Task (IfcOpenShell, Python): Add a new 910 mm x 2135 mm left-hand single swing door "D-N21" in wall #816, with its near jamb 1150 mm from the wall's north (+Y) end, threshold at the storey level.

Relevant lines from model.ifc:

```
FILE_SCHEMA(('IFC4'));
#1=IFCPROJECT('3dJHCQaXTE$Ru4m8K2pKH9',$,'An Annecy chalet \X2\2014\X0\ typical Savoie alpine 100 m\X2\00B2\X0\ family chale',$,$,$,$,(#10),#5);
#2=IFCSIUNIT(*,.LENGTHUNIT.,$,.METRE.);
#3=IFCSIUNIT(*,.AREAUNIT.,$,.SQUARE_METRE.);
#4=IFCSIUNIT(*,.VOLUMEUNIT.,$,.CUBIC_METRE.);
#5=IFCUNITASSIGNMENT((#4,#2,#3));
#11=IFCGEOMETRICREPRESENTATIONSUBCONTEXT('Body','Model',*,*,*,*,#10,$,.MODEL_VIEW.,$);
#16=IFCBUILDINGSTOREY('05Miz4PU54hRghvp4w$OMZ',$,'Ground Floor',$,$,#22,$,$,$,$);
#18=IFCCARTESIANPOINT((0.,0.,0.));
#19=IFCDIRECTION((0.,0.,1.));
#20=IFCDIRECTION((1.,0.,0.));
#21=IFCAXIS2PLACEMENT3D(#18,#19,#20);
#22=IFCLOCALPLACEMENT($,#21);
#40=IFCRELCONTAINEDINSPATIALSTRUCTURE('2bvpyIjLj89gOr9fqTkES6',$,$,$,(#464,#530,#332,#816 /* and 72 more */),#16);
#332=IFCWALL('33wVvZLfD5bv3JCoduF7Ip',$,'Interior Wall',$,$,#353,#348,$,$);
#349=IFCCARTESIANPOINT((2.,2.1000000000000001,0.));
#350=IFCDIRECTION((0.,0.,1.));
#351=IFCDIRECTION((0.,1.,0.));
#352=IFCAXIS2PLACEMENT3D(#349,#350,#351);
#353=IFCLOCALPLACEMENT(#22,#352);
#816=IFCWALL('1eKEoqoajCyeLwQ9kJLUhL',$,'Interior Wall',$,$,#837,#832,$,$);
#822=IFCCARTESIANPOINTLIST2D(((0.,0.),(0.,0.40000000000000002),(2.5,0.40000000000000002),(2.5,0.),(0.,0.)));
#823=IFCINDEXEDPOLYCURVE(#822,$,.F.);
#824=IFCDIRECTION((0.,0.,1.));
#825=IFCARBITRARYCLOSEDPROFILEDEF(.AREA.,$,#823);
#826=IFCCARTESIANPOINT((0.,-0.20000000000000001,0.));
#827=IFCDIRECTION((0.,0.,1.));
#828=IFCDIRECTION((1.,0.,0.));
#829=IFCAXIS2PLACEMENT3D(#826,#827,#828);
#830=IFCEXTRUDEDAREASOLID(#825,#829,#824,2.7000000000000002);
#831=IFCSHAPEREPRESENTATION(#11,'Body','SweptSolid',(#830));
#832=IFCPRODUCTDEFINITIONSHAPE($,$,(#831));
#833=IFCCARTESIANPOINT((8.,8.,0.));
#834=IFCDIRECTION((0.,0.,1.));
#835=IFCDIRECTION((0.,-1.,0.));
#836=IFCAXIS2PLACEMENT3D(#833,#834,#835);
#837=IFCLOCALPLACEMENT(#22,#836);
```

```python
import numpy as np
import ifcopenshell
import ifcopenshell.api.feature
import ifcopenshell.api.geometry
import ifcopenshell.api.root
import ifcopenshell.api.spatial
import ifcopenshell.geom
import ifcopenshell.util.element
import ifcopenshell.util.placement
import ifcopenshell.util.representation
import ifcopenshell.util.shape
import ifcopenshell.util.unit

model = ifcopenshell.open("model.ifc")
unit_scale = ifcopenshell.util.unit.calculate_unit_scale(model)
settings = ifcopenshell.geom.settings()


def volume(element):
    """Net volume in cubic metres, openings subtracted."""
    shape = ifcopenshell.geom.create_shape(settings, element)
    return ifcopenshell.util.shape.get_volume(shape.geometry)


wall = model.by_guid("1eKEoqoajCyeLwQ9kJLUhL")
storey = ifcopenshell.util.element.get_container(wall, ifc_class="IfcBuildingStorey")
context = ifcopenshell.util.representation.get_context(model, "Model", "Body", "MODEL_VIEW")
before = volume(wall)

width, height, from_end, sill = 0.91, 2.135, 1.15, 0.0  # metres

# The wall runs along its own X axis, and the end named is its -X end.
wall_shape = ifcopenshell.geom.create_shape(settings, wall)
x, y, z = ifcopenshell.util.shape.get_vertices(wall_shape.geometry).T
start = x.min() + from_end
face, thickness = float(y.min()), float(y.max() - y.min())
wall_matrix = ifcopenshell.util.placement.get_local_placement(wall.ObjectPlacement)
level = ifcopenshell.util.placement.get_local_placement(storey.ObjectPlacement)[2, 3]


def in_wall(x, y):
    """Placement at x, y metres in the wall's axes, at sill height."""
    matrix = wall_matrix.copy()
    matrix[:, 3] = wall_matrix @ np.array([x / unit_scale, y / unit_scale, 0.0, 1.0])
    matrix[2, 3] = level + sill / unit_scale
    return matrix


# Opening: a box that overshoots both wall faces by 50 mm.
opening = ifcopenshell.api.root.create_entity(model, ifc_class="IfcOpeningElement", predefined_type="OPENING")
box = ifcopenshell.api.geometry.add_wall_representation(
    model, context=context, length=width, height=height, thickness=thickness + 0.1
)
ifcopenshell.api.geometry.assign_representation(model, product=opening, representation=box)
ifcopenshell.api.geometry.edit_object_placement(model, product=opening, matrix=in_wall(start, face - 0.05), is_si=False)
ifcopenshell.api.feature.add_feature(model, feature=opening, element=wall)

door = ifcopenshell.api.root.create_entity(model, ifc_class="IfcDoor", name="D-N21", predefined_type="DOOR")
door.OverallWidth, door.OverallHeight = width / unit_scale, height / unit_scale
door.OperationType = "SINGLE_SWING_LEFT"
body = ifcopenshell.api.geometry.add_door_representation(
    model,
    context=context,
    overall_width=door.OverallWidth,
    overall_height=door.OverallHeight,
    operation_type="SINGLE_SWING_LEFT",
    lining_properties={"LiningDepth": thickness / unit_scale, "ThresholdDepth": thickness / unit_scale},
)
ifcopenshell.api.geometry.assign_representation(model, product=door, representation=body)
ifcopenshell.api.spatial.assign_container(model, products=[door], relating_structure=storey)
ifcopenshell.api.feature.add_filling(model, opening=opening, element=door)

# The lining spans the wall, so the door starts at the wall face.
ifcopenshell.api.geometry.edit_object_placement(model, product=door, matrix=in_wall(start, face), is_si=False)

after = volume(wall)

print(f"wall volume {before:.3f} -> {after:.3f} m3")

model.write("model-out.ifc")
```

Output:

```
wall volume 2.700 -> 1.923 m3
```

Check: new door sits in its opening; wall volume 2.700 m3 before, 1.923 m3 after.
